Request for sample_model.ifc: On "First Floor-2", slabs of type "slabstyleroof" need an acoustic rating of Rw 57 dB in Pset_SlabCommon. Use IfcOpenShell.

First a look at what the model holds.

```python
import ifcopenshell
import ifcopenshell.util.element

model = ifcopenshell.open("sample_model.ifc")
print(model.schema)
storey = next(s for s in model.by_type("IfcBuildingStorey") if s.Name == "First Floor-2")
slabs = [e for e in ifcopenshell.util.element.get_decomposition(storey) if e.is_a("IfcSlab")]
seen = {}
for e in slabs:
    element_type = ifcopenshell.util.element.get_type(e)
    key = (element_type.Name if element_type != e and element_type else None, ifcopenshell.util.element.get_pset(e, "Pset_SlabCommon", "AcousticRating"))
    seen[key] = seen.get(key, 0) + 1
for (name, value), count in sorted(seen.items(), key=str):
    print(count, "x", name, "|", value)
```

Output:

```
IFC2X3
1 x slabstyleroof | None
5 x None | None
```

```python
import ifcopenshell
import ifcopenshell.api.pset
import ifcopenshell.util.element

model = ifcopenshell.open("sample_model.ifc")

storey = next(s for s in model.by_type("IfcBuildingStorey") if s.Name == "First Floor-2")
slabs = [e for e in ifcopenshell.util.element.get_decomposition(storey) if e.is_a("IfcSlab")]

count = 0
for e in slabs:
    element_type = ifcopenshell.util.element.get_type(e)
    if element_type in (None, e) or element_type.Name != "slabstyleroof":
        continue
    # add_pset returns the element's existing set when there is one.
    pset = ifcopenshell.api.pset.add_pset(model, product=e, name="Pset_SlabCommon")
    ifcopenshell.api.pset.edit_pset(model, pset=pset, properties={"AcousticRating": "Rw 57 dB"})
    count += 1

print(count, "slabs updated")

model.write("sample_model_rev.ifc")
```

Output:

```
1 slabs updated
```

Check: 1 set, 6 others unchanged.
